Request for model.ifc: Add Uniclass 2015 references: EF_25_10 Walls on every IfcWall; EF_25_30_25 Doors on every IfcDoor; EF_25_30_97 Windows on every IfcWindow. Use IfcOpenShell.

First a look at what the model holds.

```python
import ifcopenshell

model = ifcopenshell.open("model.ifc")
print(model.schema)
print("classifications:", [c.Name for c in model.by_type("IfcClassification")])
for ifc_class in ("IfcDoor", "IfcRoof", "IfcStair", "IfcWall", "IfcWindow"):
    print(ifc_class, len(model.by_type(ifc_class)))
```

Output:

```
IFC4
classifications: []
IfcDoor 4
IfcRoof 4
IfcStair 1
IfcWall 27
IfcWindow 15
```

```python
import ifcopenshell
import ifcopenshell.api.classification

model = ifcopenshell.open("model.ifc")

system = ifcopenshell.api.classification.add_classification(model, classification="Uniclass 2015")

codes = {
    "IfcWall": ("EF_25_10", "Walls"),
    "IfcDoor": ("EF_25_30_25", "Doors"),
    "IfcWindow": ("EF_25_30_97", "Windows"),
}
for ifc_class, (code, name) in codes.items():
    products = model.by_type(ifc_class)
    ifcopenshell.api.classification.add_reference(
        model, products=products, classification=system, identification=code, name=name
    )
    print(code, len(products))

model.write("model-out.ifc")
```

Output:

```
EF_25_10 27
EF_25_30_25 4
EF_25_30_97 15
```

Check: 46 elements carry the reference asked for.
